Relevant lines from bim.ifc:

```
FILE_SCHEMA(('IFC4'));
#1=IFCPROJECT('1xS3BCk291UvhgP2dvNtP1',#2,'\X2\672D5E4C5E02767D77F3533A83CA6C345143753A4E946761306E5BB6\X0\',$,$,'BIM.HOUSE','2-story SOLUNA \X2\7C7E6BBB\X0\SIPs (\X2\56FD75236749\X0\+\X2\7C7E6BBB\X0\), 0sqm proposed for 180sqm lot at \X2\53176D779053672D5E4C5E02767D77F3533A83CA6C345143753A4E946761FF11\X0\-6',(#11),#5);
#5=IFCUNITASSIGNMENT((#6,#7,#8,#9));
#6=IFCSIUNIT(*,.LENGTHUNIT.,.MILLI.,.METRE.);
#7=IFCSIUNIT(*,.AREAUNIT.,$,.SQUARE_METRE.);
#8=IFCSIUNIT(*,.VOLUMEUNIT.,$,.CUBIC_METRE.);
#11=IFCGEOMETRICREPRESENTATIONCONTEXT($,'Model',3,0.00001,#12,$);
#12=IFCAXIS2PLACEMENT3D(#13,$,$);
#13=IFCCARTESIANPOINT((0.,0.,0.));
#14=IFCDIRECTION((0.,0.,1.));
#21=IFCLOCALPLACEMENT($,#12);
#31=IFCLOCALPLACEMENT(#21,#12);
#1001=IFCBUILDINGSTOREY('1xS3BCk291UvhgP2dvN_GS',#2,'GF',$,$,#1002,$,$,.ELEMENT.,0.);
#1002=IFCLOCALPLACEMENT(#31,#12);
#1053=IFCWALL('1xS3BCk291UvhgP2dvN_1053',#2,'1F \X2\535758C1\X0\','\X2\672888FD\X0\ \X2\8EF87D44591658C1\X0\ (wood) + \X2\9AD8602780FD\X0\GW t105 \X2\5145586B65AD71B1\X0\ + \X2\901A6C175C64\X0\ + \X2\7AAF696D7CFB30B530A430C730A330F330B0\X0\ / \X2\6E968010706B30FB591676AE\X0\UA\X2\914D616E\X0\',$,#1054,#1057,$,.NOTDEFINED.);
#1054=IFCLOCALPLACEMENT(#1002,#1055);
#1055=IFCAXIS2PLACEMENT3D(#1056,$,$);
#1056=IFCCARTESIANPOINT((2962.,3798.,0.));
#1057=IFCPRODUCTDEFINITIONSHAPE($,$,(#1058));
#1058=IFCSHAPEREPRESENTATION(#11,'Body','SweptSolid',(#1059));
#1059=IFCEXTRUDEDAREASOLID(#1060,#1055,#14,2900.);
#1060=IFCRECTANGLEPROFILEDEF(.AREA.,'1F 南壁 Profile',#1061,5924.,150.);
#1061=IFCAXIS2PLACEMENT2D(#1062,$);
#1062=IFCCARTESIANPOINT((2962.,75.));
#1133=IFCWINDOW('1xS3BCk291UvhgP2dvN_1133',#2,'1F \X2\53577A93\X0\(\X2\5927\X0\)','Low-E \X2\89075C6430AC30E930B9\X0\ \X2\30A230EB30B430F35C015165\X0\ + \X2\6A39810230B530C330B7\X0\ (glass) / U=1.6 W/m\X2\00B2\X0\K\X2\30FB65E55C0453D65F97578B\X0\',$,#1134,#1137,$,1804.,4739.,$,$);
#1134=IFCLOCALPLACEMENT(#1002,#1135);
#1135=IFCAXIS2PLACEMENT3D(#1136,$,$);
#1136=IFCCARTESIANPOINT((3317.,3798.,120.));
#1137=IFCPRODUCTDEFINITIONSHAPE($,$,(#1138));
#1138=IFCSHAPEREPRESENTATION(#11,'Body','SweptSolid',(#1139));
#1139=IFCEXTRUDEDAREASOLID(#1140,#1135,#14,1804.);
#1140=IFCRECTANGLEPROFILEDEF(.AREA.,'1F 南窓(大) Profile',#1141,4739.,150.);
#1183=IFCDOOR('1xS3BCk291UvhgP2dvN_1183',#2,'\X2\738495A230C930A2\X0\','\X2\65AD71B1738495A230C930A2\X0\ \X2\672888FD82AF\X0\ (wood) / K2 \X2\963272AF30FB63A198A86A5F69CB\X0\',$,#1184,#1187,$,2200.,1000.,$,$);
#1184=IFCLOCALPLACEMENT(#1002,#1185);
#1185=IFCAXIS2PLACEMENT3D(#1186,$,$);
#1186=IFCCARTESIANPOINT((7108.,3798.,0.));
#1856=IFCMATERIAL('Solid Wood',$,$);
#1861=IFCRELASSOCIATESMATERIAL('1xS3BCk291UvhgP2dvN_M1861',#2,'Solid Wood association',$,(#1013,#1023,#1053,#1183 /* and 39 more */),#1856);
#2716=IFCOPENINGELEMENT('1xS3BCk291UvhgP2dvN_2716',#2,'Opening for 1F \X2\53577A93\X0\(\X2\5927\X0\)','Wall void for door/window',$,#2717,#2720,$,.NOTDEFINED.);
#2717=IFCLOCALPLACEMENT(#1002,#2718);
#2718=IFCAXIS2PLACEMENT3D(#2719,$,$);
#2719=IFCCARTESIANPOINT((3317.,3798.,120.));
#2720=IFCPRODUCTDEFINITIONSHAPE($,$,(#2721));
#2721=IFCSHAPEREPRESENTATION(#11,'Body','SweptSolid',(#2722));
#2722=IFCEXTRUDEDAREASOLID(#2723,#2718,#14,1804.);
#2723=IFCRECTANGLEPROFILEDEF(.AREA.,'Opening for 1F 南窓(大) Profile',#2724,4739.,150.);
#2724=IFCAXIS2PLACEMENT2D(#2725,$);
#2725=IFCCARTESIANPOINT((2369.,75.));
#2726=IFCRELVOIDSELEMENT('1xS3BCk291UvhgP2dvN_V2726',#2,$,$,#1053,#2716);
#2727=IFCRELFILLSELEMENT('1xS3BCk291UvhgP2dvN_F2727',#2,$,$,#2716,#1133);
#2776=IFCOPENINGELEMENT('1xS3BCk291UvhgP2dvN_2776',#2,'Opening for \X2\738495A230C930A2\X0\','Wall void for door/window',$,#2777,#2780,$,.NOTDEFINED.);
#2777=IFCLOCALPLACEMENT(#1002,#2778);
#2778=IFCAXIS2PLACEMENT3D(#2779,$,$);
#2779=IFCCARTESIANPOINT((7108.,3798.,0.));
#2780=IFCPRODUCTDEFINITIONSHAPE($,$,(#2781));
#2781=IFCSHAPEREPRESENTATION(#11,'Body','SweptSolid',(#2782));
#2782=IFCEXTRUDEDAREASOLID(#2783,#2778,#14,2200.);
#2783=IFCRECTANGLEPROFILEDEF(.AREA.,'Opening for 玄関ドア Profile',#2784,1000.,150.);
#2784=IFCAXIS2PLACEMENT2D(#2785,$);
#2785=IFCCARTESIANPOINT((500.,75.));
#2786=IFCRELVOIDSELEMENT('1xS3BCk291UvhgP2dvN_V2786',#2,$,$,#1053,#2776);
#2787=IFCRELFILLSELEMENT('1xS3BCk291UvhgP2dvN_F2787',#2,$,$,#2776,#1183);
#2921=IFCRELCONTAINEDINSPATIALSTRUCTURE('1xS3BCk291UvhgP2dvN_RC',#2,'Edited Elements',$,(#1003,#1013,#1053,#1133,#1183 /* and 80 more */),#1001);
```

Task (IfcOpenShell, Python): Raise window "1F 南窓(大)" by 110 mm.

```python
import numpy as np
import ifcopenshell
import ifcopenshell.api.geometry
import ifcopenshell.util.placement
import ifcopenshell.util.unit

model = ifcopenshell.open("bim.ifc")
unit_scale = ifcopenshell.util.unit.calculate_unit_scale(model)

window = model.by_guid("1xS3BCk291UvhgP2dvN_1133")
opening = window.FillsVoids[0].RelatingOpeningElement
dz = 110.0

shift = np.array([0.0, 0.0, dz])
# The window is not placed relative to its opening, so move both.
for product in (opening, window):
    matrix = ifcopenshell.util.placement.get_local_placement(product.ObjectPlacement)
    matrix[:3, 3] += shift
    ifcopenshell.api.geometry.edit_object_placement(model, product=product, matrix=matrix, is_si=False)

print(f"moved by {dz * unit_scale:+.3f} m")

model.write("bim_updated.ifc")
```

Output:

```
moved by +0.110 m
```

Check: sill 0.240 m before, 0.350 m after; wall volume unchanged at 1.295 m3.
